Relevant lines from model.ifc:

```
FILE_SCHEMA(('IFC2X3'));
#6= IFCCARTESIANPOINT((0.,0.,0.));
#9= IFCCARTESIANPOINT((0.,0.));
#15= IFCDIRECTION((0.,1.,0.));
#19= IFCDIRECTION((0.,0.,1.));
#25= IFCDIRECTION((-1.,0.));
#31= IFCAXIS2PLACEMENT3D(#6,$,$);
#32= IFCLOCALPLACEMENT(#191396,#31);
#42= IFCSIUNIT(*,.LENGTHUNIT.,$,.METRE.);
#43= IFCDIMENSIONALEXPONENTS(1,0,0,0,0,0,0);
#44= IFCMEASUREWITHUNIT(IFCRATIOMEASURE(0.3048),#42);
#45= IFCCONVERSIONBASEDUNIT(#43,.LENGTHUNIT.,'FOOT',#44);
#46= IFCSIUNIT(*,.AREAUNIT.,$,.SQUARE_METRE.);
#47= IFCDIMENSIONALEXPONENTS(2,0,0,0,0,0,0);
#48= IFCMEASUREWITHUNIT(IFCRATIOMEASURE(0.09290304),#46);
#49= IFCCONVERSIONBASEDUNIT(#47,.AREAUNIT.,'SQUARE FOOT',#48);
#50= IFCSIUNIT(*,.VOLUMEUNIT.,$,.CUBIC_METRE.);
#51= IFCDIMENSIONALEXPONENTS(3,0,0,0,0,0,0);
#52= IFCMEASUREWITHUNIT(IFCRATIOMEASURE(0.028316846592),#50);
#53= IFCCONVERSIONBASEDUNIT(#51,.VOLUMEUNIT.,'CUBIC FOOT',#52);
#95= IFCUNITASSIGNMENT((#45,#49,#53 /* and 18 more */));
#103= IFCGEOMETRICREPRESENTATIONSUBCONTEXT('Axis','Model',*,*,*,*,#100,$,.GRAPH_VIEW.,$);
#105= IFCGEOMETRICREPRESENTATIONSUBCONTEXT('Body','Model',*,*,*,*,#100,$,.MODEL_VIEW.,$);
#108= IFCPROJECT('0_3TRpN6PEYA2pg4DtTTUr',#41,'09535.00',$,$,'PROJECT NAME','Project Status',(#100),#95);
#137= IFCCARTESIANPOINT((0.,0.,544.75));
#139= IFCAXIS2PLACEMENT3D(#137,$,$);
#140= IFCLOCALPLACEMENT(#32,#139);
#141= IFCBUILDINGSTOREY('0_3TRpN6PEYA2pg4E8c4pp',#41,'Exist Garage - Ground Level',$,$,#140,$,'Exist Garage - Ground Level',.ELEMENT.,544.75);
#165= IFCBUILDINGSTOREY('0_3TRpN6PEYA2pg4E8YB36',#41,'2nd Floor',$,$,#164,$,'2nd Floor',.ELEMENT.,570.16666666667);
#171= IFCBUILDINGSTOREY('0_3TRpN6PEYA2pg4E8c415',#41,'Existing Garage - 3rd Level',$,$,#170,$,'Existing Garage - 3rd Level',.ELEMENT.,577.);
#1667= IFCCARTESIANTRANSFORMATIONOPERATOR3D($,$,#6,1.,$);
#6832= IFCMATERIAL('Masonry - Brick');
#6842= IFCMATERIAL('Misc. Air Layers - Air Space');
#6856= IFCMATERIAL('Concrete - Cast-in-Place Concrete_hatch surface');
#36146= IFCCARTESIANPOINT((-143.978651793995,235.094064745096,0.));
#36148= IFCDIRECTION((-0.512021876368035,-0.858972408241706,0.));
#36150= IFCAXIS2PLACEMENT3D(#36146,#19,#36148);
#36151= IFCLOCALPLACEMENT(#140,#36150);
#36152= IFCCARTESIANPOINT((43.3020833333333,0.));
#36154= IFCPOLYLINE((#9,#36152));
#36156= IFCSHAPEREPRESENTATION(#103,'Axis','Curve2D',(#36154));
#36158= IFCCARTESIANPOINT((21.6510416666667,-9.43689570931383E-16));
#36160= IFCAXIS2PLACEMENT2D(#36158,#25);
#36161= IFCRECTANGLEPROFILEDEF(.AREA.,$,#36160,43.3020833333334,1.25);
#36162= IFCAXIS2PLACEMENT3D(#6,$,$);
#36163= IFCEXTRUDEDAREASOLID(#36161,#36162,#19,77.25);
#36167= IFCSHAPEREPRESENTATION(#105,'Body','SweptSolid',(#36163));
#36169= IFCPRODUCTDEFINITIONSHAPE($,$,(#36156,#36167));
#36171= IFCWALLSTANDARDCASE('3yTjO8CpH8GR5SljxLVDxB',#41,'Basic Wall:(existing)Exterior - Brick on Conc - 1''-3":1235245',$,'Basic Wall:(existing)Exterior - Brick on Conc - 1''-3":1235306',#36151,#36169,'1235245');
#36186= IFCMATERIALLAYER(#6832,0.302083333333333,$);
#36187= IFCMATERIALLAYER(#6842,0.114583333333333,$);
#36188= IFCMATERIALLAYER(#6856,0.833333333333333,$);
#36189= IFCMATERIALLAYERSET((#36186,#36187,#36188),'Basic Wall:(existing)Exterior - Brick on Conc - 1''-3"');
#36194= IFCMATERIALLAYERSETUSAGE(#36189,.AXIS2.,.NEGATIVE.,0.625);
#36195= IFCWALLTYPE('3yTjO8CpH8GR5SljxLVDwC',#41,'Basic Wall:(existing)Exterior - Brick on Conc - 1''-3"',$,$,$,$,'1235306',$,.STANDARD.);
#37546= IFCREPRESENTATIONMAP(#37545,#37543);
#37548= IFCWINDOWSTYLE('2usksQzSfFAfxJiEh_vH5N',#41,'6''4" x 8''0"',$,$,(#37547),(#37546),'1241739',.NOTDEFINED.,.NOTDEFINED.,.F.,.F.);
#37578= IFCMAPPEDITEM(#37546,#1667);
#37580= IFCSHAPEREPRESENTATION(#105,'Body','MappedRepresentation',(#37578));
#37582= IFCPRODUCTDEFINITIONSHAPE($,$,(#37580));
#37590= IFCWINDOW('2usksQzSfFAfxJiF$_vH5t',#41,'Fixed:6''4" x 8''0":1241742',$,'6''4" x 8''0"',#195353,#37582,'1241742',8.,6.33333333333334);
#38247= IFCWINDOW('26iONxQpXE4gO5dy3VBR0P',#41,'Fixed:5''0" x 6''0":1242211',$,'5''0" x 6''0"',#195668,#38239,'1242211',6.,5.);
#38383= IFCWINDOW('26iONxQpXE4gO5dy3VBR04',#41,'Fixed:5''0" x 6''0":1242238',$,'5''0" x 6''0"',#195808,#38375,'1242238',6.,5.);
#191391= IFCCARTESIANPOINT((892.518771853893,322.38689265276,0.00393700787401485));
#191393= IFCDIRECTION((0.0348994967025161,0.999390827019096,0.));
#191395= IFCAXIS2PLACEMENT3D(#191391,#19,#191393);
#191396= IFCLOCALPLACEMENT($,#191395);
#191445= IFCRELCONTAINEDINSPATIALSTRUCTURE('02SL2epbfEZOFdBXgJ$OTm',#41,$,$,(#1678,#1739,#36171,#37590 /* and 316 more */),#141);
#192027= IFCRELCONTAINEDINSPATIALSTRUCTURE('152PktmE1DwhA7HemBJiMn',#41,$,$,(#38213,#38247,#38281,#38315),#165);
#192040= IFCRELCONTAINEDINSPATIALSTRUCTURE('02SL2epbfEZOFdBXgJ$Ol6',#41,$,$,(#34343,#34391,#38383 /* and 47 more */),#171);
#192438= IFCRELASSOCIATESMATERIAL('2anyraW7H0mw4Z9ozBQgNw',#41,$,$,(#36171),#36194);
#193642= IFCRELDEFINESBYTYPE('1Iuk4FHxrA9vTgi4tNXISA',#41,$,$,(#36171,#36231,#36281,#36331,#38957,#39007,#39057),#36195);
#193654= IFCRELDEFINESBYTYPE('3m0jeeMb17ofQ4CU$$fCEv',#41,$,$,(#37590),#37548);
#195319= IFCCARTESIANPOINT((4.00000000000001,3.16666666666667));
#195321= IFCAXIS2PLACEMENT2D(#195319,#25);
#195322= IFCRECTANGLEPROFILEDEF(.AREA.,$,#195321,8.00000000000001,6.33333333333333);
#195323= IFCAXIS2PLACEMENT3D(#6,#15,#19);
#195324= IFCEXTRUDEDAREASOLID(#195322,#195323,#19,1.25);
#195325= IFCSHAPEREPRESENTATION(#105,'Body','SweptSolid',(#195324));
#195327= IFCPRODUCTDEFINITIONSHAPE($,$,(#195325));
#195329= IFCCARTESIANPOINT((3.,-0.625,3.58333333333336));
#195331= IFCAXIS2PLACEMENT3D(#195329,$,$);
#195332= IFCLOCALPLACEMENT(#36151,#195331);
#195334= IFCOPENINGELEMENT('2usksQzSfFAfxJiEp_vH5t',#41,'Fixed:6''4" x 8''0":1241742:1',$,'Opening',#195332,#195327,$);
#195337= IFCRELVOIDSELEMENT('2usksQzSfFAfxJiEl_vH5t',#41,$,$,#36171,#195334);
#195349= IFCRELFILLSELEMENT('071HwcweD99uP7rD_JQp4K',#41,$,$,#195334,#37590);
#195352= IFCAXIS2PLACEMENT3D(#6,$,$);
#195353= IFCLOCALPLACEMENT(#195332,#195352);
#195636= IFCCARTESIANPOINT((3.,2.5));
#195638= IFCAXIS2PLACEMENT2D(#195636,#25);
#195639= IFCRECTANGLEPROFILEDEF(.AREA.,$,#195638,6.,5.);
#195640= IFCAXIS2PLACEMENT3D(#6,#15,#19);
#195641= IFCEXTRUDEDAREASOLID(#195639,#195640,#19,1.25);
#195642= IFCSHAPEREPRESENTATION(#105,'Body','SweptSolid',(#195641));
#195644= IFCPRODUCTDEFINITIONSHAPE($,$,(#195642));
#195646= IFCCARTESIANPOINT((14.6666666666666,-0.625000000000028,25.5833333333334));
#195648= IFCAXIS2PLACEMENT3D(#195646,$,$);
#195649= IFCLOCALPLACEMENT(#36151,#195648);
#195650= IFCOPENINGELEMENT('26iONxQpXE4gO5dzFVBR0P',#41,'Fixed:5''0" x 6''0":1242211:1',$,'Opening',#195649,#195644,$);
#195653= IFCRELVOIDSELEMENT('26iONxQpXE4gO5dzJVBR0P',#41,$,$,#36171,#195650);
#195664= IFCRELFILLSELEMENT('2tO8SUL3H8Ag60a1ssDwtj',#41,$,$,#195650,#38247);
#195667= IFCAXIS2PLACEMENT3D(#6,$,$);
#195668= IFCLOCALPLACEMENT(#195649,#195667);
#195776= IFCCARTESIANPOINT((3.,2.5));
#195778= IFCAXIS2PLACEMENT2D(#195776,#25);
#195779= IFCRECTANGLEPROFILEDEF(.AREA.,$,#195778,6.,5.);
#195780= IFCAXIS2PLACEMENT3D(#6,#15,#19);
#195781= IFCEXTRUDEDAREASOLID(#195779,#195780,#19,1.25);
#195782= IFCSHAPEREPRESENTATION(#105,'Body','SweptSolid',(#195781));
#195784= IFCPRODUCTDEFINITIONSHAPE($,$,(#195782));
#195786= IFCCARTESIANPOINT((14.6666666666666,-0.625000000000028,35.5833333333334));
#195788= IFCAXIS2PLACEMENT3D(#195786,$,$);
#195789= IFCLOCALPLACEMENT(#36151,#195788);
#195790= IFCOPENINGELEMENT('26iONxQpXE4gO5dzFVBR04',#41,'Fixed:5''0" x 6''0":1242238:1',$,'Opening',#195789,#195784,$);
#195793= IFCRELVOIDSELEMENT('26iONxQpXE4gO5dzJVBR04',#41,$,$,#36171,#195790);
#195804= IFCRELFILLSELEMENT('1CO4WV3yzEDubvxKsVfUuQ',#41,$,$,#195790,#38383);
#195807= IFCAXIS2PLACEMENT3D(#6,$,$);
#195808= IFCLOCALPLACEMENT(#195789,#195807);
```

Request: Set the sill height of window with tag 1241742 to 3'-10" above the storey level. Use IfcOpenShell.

```python
import numpy as np
import ifcopenshell
import ifcopenshell.api.geometry
import ifcopenshell.geom
import ifcopenshell.util.element
import ifcopenshell.util.placement
import ifcopenshell.util.shape
import ifcopenshell.util.unit

model = ifcopenshell.open("model.ifc")
unit_scale = ifcopenshell.util.unit.calculate_unit_scale(model)

window = model.by_guid("2usksQzSfFAfxJiF$_vH5t")
opening = window.FillsVoids[0].RelatingOpeningElement
storey = ifcopenshell.util.element.get_container(window, ifc_class="IfcBuildingStorey")
level = ifcopenshell.util.placement.get_local_placement(storey.ObjectPlacement)[2, 3]

# The opening's origin need not be at the sill, so measure its lowest point.
shape = ifcopenshell.geom.create_shape(ifcopenshell.geom.settings(), opening)
bottom = ifcopenshell.util.shape.get_shape_bottom_elevation(shape, shape.geometry) / unit_scale
dz = level + 46 * 0.0254 / unit_scale - bottom

shift = np.array([0.0, 0.0, dz])
# The window is placed relative to its opening, so it follows when the opening moves.
matrix = ifcopenshell.util.placement.get_local_placement(opening.ObjectPlacement)
matrix[:3, 3] += shift
ifcopenshell.api.geometry.edit_object_placement(
    model, product=opening, matrix=matrix, is_si=False, should_transform_children=True
)

print(f"moved by {dz * unit_scale:+.3f} m")

model.write("model_updated.ifc")
```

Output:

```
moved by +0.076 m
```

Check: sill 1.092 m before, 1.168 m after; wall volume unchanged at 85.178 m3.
